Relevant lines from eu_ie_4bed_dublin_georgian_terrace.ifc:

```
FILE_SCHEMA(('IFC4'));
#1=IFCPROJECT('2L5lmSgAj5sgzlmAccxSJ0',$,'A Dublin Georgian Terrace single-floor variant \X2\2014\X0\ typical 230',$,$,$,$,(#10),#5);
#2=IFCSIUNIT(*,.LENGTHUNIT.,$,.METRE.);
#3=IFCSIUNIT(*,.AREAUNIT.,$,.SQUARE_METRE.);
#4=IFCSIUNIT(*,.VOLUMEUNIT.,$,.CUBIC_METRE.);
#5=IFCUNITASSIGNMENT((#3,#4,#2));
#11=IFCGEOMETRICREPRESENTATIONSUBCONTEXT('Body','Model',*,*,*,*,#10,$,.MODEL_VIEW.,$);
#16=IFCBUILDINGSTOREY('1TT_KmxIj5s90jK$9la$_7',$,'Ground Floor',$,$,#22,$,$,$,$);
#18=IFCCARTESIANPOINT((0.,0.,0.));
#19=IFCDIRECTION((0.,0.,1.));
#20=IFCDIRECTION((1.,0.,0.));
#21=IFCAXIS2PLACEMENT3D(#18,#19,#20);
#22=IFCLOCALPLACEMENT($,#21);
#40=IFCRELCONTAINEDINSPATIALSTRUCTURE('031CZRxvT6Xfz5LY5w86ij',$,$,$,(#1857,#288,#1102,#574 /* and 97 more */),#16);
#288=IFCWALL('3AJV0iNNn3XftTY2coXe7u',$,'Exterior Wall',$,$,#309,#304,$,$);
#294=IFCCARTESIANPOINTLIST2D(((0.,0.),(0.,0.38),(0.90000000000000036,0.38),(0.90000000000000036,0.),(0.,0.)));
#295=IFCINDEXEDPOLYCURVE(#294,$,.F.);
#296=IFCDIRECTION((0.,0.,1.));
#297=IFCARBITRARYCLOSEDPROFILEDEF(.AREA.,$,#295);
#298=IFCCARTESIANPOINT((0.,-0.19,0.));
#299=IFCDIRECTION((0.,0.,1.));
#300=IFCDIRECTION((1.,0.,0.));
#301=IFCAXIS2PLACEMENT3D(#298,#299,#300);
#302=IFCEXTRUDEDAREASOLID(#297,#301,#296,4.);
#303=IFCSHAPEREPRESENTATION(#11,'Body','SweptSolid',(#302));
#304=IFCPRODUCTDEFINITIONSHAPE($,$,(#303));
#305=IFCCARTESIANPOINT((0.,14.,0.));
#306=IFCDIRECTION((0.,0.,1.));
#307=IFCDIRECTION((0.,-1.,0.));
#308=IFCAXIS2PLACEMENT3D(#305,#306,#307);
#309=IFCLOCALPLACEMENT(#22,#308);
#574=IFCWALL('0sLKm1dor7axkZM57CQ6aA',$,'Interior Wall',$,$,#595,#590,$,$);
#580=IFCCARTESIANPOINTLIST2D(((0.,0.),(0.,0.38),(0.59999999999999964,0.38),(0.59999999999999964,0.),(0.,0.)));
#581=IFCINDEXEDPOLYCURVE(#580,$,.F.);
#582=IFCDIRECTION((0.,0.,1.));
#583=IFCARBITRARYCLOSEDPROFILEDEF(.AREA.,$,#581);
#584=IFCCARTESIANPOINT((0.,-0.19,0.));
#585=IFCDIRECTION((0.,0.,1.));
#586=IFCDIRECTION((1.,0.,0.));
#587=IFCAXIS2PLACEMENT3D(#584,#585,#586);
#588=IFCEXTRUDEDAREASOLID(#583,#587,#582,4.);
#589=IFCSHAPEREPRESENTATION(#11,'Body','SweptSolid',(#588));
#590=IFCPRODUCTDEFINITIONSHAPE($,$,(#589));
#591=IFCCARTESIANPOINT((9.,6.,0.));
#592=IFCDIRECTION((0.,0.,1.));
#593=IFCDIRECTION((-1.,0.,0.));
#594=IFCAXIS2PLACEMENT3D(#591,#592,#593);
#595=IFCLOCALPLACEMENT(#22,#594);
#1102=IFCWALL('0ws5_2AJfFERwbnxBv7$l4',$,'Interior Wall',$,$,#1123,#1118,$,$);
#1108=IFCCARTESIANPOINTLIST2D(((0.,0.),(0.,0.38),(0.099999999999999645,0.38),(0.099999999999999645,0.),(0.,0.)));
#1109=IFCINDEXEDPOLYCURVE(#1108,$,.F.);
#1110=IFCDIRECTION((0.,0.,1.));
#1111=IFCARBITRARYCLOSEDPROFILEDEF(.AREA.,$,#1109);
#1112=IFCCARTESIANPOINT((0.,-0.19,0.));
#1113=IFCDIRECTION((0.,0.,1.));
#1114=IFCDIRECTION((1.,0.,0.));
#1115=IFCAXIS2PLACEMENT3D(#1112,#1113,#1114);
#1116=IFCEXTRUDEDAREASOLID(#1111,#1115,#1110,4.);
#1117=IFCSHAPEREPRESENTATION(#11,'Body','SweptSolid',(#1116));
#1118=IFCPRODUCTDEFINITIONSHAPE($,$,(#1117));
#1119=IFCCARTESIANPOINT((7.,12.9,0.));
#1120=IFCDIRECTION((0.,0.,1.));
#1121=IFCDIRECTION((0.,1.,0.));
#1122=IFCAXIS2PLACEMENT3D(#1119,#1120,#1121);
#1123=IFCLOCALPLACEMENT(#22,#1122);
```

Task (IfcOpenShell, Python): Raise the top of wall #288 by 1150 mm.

```python
import ifcopenshell
import ifcopenshell.geom
import ifcopenshell.util.representation
import ifcopenshell.util.shape

model = ifcopenshell.open("eu_ie_4bed_dublin_georgian_terrace.ifc")
settings = ifcopenshell.geom.settings()


def volume(element):
    """Net volume in cubic metres, openings subtracted."""
    shape = ifcopenshell.geom.create_shape(settings, element)
    return ifcopenshell.util.shape.get_volume(shape.geometry)


wall = model.by_id(288)
before = volume(wall)

body = ifcopenshell.util.representation.get_representation(wall, "Model", "Body")
solid = body.Items[0]
old_height = solid.Depth
solid.Depth += 1.15
after = volume(wall)

print(f"height {old_height:g} -> {solid.Depth:g}, volume {before:.3f} -> {after:.3f} m3")

model.write("eu_ie_4bed_dublin_georgian_terrace_updated.ifc")
```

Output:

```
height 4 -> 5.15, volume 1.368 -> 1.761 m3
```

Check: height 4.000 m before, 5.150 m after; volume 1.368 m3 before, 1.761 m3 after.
